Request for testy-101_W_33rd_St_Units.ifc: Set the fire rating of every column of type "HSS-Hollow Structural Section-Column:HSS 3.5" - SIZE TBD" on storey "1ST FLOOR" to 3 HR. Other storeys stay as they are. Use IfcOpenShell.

First a look at what the model holds.

```python
import ifcopenshell
import ifcopenshell.util.element

model = ifcopenshell.open("testy-101_W_33rd_St_Units.ifc")
print(model.schema)
storey = next(s for s in model.by_type("IfcBuildingStorey") if s.Name == "1ST FLOOR")
columns = [e for e in ifcopenshell.util.element.get_decomposition(storey) if e.is_a("IfcColumn")]
seen = {}
for e in columns:
    element_type = ifcopenshell.util.element.get_type(e)
    key = (element_type.Name if element_type != e and element_type else None, ifcopenshell.util.element.get_pset(e, "Pset_ColumnCommon", "FireRating"))
    seen[key] = seen.get(key, 0) + 1
for (name, value), count in sorted(seen.items(), key=str):
    print(count, "x", name, "|", value)
```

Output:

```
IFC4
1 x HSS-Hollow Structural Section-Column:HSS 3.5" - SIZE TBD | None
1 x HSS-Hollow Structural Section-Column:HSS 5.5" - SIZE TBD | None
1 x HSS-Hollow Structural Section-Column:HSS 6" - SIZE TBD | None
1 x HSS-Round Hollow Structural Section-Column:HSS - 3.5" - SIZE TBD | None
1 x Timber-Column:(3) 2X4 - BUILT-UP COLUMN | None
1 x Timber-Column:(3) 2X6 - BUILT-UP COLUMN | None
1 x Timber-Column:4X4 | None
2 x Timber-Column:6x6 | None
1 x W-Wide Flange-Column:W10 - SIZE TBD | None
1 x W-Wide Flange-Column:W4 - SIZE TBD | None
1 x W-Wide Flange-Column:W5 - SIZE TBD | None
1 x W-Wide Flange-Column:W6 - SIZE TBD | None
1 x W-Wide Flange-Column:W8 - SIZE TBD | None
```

```python
import ifcopenshell
import ifcopenshell.api.pset
import ifcopenshell.util.element

model = ifcopenshell.open("testy-101_W_33rd_St_Units.ifc")

storey = next(s for s in model.by_type("IfcBuildingStorey") if s.Name == "1ST FLOOR")
columns = [e for e in ifcopenshell.util.element.get_decomposition(storey) if e.is_a("IfcColumn")]

count = 0
for e in columns:
    element_type = ifcopenshell.util.element.get_type(e)
    if element_type in (None, e) or element_type.Name != 'HSS-Hollow Structural Section-Column:HSS 3.5" - SIZE TBD':
        continue
    # add_pset returns the element's existing set when there is one.
    pset = ifcopenshell.api.pset.add_pset(model, product=e, name="Pset_ColumnCommon")
    ifcopenshell.api.pset.edit_pset(model, pset=pset, properties={"FireRating": "3 HR"})
    count += 1

print(count, "columns updated")

model.write("testy-101_W_33rd_St_Units_rev.ifc")
```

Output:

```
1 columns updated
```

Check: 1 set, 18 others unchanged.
